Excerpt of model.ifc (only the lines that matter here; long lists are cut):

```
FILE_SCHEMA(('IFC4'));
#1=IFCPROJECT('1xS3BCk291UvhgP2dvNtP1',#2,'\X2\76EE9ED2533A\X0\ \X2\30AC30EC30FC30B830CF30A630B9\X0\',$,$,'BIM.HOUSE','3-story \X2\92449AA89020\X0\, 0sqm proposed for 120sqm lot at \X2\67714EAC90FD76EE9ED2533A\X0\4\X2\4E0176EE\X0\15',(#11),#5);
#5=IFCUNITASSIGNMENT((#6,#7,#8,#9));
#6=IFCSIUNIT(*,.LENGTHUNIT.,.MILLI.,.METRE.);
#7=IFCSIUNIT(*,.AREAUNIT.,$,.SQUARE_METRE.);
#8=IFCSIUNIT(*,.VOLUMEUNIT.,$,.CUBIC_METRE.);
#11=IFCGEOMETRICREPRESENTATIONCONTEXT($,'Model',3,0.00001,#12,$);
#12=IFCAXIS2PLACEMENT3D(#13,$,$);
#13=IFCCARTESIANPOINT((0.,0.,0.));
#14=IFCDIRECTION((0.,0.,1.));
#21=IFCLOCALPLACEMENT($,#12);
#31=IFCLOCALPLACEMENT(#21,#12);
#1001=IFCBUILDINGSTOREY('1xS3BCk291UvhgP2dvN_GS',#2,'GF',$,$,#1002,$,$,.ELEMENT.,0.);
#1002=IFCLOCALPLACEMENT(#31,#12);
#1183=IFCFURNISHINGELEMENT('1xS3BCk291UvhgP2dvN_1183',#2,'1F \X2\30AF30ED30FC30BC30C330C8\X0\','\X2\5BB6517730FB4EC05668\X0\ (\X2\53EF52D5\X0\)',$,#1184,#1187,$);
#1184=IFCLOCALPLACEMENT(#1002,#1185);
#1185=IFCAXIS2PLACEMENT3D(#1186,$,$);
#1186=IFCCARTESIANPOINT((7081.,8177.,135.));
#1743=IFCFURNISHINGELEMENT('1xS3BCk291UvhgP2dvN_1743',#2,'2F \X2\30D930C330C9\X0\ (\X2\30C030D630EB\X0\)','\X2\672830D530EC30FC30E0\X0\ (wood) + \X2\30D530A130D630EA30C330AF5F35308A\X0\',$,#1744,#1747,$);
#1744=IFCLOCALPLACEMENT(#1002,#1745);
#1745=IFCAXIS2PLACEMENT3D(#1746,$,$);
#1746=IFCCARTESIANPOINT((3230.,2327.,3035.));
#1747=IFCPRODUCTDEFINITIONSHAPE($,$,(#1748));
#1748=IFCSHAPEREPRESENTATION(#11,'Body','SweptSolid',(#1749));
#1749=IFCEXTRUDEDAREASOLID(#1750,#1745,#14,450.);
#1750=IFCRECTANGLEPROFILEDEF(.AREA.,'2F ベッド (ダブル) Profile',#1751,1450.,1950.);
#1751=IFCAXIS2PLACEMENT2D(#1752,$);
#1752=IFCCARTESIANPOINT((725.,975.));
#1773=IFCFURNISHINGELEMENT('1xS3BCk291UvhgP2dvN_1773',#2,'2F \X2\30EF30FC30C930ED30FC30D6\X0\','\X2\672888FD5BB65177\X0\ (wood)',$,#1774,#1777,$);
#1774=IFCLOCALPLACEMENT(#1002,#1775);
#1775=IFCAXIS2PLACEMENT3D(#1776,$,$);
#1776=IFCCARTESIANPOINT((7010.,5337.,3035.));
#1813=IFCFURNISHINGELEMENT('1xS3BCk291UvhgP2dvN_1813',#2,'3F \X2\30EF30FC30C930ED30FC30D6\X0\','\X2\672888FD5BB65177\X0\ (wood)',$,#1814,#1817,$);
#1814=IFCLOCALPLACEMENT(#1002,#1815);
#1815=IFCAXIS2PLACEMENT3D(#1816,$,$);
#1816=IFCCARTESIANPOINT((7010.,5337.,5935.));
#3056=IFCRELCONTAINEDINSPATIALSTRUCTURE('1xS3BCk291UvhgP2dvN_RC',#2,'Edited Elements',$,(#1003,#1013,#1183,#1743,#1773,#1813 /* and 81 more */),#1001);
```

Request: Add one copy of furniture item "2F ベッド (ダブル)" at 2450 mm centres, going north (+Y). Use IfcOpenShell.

```python
import numpy as np
import ifcopenshell
import ifcopenshell.api.geometry
import ifcopenshell.api.root
import ifcopenshell.util.element
import ifcopenshell.util.placement
import ifcopenshell.util.unit

model = ifcopenshell.open("model.ifc")
unit_scale = ifcopenshell.util.unit.calculate_unit_scale(model)


def reuse_history(source, copy):
    """copy_class also copies each property set's owner history, people and application; keep the originals."""
    for rel in copy.IsDefinedBy:
        if rel.is_a("IfcRelDefinesByProperties") and (history := rel.RelatingPropertyDefinition.OwnerHistory):
            rel.RelatingPropertyDefinition.OwnerHistory = source.OwnerHistory
            ifcopenshell.util.element.remove_deep2(model, history)


source = model.by_guid("1xS3BCk291UvhgP2dvN_1743")
base = ifcopenshell.util.placement.get_local_placement(source.ObjectPlacement)
step = np.array([0.0, 1.0, 0.0]) * 2.45 / unit_scale

for i in range(1, 2):
    copy = ifcopenshell.api.root.copy_class(model, product=source)
    copy.Representation = ifcopenshell.util.element.copy_deep(
        model, source.Representation, exclude=["IfcGeometricRepresentationContext", "IfcRepresentationMap"]
    )
    reuse_history(source, copy)
    matrix = base.copy()
    matrix[:3, 3] += i * step
    print("added at", matrix[:3, 3].round(3) + 0.0)
    ifcopenshell.api.geometry.edit_object_placement(model, product=copy, matrix=matrix, is_si=False)

model.write("model-out.ifc")
```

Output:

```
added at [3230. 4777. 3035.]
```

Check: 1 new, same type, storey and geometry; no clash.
